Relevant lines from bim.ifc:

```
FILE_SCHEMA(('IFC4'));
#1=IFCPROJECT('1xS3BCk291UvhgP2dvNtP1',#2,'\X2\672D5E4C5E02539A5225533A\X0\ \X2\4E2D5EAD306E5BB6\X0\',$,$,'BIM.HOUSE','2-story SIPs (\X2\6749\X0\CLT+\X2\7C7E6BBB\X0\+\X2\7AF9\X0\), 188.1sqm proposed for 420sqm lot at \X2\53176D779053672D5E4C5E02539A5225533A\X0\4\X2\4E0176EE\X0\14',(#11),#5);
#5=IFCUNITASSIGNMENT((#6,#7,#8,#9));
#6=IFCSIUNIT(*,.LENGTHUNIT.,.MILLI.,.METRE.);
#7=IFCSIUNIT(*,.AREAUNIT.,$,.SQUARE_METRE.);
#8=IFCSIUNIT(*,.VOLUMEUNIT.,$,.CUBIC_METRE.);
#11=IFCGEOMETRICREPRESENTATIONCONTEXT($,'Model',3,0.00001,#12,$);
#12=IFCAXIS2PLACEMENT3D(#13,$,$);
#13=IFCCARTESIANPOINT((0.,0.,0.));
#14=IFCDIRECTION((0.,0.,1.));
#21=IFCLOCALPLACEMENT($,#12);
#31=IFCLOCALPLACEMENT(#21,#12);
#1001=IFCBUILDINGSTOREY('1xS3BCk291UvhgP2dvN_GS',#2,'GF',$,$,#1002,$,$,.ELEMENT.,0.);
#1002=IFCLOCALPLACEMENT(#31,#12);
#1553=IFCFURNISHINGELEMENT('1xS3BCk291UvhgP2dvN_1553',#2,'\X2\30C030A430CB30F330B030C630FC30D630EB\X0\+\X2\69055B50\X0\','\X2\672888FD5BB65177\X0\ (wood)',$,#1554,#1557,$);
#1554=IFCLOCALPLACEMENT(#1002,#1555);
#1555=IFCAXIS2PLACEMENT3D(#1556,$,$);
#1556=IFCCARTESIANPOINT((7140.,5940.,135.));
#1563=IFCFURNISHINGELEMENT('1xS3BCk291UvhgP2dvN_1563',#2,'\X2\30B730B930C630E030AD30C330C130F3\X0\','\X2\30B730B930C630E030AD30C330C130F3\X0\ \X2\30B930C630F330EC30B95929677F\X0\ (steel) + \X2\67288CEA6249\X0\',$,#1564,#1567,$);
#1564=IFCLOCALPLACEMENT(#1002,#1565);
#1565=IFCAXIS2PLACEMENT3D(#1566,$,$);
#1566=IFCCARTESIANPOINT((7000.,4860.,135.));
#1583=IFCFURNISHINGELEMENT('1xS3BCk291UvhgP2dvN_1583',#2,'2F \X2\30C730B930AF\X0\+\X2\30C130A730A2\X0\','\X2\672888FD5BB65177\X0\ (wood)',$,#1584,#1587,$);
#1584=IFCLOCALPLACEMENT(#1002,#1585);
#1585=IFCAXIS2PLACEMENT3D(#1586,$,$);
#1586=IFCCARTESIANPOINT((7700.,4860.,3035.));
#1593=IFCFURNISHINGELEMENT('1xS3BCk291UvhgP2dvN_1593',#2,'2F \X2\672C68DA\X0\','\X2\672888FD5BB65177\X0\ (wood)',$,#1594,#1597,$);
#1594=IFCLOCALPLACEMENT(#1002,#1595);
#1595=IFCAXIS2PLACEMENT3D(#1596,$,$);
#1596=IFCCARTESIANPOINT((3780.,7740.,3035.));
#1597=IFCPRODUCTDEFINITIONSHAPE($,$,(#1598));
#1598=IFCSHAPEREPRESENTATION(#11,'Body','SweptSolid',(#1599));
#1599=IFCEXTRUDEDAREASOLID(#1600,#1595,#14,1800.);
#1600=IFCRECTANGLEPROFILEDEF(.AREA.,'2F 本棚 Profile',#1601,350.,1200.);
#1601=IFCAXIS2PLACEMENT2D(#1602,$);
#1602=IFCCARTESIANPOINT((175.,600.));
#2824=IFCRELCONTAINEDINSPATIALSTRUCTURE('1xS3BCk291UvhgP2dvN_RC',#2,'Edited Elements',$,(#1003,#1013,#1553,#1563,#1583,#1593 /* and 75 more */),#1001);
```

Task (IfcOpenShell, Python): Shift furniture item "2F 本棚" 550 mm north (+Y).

```python
import ifcopenshell
import ifcopenshell.api.geometry
import ifcopenshell.util.placement
import ifcopenshell.util.unit

model = ifcopenshell.open("bim.ifc")
unit_scale = ifcopenshell.util.unit.calculate_unit_scale(model)

item = model.by_guid("1xS3BCk291UvhgP2dvN_1593")
matrix = ifcopenshell.util.placement.get_local_placement(item.ObjectPlacement)
matrix[1, 3] += 0.55 / unit_scale
ifcopenshell.api.geometry.edit_object_placement(model, product=item, matrix=matrix, is_si=False)

print(ifcopenshell.util.placement.get_local_placement(item.ObjectPlacement).round(3) + 0.0)

model.write("bim_updated.ifc")
```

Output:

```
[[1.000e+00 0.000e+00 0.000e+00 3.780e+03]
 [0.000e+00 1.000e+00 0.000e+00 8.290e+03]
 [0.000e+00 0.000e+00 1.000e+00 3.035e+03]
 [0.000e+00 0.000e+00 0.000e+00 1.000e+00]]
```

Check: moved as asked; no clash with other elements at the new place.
